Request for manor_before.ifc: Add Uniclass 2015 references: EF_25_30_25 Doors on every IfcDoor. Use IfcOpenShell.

First a look at what the model holds.

```python
import ifcopenshell

model = ifcopenshell.open("manor_before.ifc")
print(model.schema)
print("classifications:", [c.Name for c in model.by_type("IfcClassification")])
for ifc_class in ("IfcDoor", "IfcRoof", "IfcStair", "IfcWall", "IfcWindow"):
    print(ifc_class, len(model.by_type(ifc_class)))
```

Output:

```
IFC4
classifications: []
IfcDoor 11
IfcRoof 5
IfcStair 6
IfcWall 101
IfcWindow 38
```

```python
import ifcopenshell
import ifcopenshell.api.classification

model = ifcopenshell.open("manor_before.ifc")

system = ifcopenshell.api.classification.add_classification(model, classification="Uniclass 2015")

codes = {
    "IfcDoor": ("EF_25_30_25", "Doors"),
}
for ifc_class, (code, name) in codes.items():
    products = model.by_type(ifc_class)
    ifcopenshell.api.classification.add_reference(
        model, products=products, classification=system, identification=code, name=name
    )
    print(code, len(products))

model.write("manor_before_updated.ifc")
```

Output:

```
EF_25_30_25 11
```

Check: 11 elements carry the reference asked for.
